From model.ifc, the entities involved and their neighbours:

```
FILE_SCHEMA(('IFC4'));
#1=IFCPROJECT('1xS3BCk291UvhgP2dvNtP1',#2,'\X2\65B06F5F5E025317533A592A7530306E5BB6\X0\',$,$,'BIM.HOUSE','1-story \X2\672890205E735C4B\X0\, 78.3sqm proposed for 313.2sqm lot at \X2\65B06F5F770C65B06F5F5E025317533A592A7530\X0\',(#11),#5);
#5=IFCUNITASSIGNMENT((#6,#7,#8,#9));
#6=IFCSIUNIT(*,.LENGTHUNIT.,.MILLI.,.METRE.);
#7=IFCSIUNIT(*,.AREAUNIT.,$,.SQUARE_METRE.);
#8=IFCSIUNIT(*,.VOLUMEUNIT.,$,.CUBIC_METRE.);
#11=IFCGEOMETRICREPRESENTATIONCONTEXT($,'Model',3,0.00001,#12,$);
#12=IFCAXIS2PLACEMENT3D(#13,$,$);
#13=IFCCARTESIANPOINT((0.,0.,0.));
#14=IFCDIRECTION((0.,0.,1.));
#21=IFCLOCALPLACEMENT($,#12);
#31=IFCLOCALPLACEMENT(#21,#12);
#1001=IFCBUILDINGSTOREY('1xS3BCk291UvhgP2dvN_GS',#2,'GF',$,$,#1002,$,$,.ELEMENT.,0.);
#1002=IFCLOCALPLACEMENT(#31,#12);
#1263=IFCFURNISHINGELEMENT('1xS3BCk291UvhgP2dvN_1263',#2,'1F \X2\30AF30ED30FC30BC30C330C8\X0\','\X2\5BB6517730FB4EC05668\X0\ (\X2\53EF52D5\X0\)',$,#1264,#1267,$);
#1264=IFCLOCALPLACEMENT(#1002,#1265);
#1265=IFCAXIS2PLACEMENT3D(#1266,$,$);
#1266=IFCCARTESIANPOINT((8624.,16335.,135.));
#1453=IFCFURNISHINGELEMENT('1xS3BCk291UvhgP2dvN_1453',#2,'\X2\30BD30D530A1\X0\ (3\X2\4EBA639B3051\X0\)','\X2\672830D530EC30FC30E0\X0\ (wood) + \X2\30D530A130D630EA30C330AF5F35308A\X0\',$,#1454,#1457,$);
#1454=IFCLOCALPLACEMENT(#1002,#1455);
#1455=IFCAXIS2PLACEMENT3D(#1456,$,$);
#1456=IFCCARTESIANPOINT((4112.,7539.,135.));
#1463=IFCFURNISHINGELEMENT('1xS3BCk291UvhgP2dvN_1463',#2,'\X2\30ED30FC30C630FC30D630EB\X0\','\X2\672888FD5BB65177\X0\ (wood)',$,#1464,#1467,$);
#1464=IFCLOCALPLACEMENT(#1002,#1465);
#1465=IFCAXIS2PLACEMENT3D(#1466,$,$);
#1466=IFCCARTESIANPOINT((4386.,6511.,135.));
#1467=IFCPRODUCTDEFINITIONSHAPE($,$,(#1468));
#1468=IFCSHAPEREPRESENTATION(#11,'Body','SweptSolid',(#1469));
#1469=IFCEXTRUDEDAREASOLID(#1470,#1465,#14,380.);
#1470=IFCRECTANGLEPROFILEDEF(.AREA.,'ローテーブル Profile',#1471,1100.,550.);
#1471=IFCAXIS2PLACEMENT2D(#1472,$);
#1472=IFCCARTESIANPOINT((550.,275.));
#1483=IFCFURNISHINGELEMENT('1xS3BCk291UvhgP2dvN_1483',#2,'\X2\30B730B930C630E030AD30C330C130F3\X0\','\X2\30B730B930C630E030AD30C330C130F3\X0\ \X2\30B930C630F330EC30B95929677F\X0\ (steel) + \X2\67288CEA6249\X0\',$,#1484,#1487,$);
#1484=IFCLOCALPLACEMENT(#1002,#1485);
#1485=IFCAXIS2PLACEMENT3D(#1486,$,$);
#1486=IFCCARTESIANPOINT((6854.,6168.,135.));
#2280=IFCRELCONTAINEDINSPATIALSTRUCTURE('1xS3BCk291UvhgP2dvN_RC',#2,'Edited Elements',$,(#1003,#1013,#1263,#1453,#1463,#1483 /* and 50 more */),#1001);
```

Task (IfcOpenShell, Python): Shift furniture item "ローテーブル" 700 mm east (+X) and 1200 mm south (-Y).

```python
import ifcopenshell
import ifcopenshell.api.geometry
import ifcopenshell.util.placement

model = ifcopenshell.open("model.ifc")

item = model.by_guid("1xS3BCk291UvhgP2dvN_1463")
matrix = ifcopenshell.util.placement.get_local_placement(item.ObjectPlacement)
matrix[0, 3] += 700.0
matrix[1, 3] -= 1200.0
ifcopenshell.api.geometry.edit_object_placement(model, product=item, matrix=matrix, is_si=False)

print(ifcopenshell.util.placement.get_local_placement(item.ObjectPlacement).round(3) + 0.0)

model.write("model_updated.ifc")
```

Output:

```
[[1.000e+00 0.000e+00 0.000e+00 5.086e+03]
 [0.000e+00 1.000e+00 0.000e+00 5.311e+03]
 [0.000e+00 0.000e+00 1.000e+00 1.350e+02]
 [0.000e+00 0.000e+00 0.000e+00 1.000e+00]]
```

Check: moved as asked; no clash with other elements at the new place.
